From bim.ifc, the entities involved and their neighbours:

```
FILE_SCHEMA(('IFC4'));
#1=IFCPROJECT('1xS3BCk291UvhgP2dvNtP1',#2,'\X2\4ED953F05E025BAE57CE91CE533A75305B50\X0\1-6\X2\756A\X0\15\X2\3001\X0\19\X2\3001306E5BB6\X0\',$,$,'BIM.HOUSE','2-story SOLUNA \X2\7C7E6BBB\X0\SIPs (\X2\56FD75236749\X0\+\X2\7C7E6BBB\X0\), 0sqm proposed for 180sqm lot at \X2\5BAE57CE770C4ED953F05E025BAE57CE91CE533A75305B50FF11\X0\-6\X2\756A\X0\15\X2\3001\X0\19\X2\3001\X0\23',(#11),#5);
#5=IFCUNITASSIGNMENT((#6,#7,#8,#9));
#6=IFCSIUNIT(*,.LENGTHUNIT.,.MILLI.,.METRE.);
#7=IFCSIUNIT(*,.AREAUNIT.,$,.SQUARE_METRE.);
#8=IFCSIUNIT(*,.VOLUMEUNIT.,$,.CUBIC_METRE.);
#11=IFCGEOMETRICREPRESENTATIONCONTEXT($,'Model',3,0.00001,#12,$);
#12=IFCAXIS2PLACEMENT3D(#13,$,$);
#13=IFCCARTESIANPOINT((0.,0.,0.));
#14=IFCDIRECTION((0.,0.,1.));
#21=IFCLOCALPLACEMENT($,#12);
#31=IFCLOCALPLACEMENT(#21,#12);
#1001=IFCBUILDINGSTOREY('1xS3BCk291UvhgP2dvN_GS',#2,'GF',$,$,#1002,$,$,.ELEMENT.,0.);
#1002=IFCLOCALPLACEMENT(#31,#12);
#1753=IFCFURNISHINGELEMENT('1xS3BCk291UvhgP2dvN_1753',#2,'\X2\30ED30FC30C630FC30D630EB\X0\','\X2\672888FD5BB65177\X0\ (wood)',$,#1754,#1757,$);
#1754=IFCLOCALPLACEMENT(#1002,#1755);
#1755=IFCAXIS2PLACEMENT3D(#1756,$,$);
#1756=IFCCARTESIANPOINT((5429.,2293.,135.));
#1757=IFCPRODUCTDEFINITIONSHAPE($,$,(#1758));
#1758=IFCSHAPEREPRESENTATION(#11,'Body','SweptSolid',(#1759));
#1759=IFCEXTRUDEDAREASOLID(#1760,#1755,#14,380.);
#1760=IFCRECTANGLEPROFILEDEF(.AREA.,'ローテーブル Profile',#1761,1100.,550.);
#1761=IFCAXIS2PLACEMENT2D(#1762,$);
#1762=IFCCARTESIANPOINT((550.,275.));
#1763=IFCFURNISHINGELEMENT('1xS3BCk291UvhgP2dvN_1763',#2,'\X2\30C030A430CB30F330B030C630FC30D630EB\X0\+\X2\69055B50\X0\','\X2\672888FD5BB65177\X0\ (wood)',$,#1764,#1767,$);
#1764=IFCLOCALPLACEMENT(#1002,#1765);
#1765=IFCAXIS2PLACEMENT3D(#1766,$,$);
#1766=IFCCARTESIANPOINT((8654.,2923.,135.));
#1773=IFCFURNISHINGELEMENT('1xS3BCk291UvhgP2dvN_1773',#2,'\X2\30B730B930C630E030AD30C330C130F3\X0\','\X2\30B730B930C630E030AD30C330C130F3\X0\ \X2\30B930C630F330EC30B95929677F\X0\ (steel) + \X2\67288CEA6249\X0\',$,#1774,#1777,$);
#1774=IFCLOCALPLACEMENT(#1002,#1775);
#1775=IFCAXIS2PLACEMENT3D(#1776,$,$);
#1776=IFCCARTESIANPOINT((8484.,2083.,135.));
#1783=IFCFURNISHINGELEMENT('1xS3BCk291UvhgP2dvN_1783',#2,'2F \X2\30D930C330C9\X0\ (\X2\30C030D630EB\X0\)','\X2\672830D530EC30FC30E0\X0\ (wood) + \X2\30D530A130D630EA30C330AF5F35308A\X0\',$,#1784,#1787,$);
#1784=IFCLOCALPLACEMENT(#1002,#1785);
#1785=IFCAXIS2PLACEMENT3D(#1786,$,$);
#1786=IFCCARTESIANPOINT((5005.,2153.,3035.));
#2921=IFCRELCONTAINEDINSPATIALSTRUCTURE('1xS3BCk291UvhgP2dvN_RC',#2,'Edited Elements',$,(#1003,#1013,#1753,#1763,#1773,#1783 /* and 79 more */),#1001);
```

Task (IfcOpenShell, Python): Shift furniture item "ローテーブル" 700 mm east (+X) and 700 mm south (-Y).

```python
import ifcopenshell
import ifcopenshell.api.geometry
import ifcopenshell.util.placement
import ifcopenshell.util.unit

model = ifcopenshell.open("bim.ifc")
unit_scale = ifcopenshell.util.unit.calculate_unit_scale(model)

item = model.by_id(1753)
matrix = ifcopenshell.util.placement.get_local_placement(item.ObjectPlacement)
matrix[0, 3] += 0.7 / unit_scale
matrix[1, 3] -= 0.7 / unit_scale
ifcopenshell.api.geometry.edit_object_placement(model, product=item, matrix=matrix, is_si=False)

print(ifcopenshell.util.placement.get_local_placement(item.ObjectPlacement).round(3) + 0.0)

model.write("bim_updated.ifc")
```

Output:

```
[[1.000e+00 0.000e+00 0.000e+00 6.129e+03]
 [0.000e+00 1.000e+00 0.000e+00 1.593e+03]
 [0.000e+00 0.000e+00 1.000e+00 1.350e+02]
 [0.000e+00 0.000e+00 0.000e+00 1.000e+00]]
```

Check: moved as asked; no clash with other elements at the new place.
